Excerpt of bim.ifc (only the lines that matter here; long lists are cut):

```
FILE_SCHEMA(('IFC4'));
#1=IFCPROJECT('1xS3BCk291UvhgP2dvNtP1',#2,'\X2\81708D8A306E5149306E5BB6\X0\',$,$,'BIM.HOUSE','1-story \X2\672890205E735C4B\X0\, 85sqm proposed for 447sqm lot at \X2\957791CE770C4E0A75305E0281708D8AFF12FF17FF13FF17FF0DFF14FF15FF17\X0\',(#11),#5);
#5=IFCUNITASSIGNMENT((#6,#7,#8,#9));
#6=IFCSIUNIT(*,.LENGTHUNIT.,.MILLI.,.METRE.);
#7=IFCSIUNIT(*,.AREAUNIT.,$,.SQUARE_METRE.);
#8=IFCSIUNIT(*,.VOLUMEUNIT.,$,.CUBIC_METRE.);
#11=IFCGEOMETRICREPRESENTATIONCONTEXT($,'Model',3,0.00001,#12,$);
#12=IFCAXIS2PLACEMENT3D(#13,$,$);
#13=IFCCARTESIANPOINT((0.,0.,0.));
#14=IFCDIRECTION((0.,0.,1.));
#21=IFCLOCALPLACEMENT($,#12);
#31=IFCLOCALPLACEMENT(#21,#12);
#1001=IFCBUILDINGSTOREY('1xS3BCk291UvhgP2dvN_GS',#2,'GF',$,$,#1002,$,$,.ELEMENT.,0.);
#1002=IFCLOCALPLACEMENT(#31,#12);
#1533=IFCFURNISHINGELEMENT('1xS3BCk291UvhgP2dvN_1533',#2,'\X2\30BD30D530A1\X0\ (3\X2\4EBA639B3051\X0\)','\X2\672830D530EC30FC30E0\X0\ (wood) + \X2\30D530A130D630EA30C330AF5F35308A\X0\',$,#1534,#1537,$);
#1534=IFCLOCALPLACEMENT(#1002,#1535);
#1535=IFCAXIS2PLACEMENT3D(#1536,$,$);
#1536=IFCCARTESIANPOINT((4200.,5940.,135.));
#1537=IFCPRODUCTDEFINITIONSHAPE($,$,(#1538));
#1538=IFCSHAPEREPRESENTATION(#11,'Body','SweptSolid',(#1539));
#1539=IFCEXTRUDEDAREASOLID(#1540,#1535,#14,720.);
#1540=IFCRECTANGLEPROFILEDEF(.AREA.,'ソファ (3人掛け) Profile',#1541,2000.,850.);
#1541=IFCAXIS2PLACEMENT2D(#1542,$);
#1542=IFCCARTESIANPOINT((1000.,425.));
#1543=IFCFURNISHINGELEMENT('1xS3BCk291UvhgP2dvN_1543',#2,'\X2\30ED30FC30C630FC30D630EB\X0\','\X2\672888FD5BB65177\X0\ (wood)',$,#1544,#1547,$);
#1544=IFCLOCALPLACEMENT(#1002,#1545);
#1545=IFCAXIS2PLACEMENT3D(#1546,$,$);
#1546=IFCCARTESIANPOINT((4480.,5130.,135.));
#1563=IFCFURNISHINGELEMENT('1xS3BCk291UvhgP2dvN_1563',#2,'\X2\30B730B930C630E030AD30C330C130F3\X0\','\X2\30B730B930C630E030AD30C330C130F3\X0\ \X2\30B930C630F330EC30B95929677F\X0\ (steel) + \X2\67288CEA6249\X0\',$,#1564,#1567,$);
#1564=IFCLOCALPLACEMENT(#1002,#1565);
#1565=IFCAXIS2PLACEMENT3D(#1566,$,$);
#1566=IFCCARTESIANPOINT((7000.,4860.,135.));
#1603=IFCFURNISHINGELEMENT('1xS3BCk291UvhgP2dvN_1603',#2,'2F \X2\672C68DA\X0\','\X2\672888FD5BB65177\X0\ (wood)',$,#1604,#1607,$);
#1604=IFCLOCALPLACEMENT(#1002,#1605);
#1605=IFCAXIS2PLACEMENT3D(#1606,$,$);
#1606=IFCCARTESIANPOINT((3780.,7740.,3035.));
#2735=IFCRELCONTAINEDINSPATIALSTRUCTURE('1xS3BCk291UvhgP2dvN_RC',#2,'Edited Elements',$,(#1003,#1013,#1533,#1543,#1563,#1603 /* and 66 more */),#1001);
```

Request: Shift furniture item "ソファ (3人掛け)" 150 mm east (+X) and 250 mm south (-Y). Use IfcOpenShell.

```python
import ifcopenshell
import ifcopenshell.api.geometry
import ifcopenshell.util.placement
import ifcopenshell.util.unit

model = ifcopenshell.open("bim.ifc")
unit_scale = ifcopenshell.util.unit.calculate_unit_scale(model)

item = model.by_guid("1xS3BCk291UvhgP2dvN_1533")
matrix = ifcopenshell.util.placement.get_local_placement(item.ObjectPlacement)
matrix[0, 3] += 0.15 / unit_scale
matrix[1, 3] -= 0.25 / unit_scale
ifcopenshell.api.geometry.edit_object_placement(model, product=item, matrix=matrix, is_si=False)

print(ifcopenshell.util.placement.get_local_placement(item.ObjectPlacement).round(3) + 0.0)

model.write("bim_rev.ifc")
```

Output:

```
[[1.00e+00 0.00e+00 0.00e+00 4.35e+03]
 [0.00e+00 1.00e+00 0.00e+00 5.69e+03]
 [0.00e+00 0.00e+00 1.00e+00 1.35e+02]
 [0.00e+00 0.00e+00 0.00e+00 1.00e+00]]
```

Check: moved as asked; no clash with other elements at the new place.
